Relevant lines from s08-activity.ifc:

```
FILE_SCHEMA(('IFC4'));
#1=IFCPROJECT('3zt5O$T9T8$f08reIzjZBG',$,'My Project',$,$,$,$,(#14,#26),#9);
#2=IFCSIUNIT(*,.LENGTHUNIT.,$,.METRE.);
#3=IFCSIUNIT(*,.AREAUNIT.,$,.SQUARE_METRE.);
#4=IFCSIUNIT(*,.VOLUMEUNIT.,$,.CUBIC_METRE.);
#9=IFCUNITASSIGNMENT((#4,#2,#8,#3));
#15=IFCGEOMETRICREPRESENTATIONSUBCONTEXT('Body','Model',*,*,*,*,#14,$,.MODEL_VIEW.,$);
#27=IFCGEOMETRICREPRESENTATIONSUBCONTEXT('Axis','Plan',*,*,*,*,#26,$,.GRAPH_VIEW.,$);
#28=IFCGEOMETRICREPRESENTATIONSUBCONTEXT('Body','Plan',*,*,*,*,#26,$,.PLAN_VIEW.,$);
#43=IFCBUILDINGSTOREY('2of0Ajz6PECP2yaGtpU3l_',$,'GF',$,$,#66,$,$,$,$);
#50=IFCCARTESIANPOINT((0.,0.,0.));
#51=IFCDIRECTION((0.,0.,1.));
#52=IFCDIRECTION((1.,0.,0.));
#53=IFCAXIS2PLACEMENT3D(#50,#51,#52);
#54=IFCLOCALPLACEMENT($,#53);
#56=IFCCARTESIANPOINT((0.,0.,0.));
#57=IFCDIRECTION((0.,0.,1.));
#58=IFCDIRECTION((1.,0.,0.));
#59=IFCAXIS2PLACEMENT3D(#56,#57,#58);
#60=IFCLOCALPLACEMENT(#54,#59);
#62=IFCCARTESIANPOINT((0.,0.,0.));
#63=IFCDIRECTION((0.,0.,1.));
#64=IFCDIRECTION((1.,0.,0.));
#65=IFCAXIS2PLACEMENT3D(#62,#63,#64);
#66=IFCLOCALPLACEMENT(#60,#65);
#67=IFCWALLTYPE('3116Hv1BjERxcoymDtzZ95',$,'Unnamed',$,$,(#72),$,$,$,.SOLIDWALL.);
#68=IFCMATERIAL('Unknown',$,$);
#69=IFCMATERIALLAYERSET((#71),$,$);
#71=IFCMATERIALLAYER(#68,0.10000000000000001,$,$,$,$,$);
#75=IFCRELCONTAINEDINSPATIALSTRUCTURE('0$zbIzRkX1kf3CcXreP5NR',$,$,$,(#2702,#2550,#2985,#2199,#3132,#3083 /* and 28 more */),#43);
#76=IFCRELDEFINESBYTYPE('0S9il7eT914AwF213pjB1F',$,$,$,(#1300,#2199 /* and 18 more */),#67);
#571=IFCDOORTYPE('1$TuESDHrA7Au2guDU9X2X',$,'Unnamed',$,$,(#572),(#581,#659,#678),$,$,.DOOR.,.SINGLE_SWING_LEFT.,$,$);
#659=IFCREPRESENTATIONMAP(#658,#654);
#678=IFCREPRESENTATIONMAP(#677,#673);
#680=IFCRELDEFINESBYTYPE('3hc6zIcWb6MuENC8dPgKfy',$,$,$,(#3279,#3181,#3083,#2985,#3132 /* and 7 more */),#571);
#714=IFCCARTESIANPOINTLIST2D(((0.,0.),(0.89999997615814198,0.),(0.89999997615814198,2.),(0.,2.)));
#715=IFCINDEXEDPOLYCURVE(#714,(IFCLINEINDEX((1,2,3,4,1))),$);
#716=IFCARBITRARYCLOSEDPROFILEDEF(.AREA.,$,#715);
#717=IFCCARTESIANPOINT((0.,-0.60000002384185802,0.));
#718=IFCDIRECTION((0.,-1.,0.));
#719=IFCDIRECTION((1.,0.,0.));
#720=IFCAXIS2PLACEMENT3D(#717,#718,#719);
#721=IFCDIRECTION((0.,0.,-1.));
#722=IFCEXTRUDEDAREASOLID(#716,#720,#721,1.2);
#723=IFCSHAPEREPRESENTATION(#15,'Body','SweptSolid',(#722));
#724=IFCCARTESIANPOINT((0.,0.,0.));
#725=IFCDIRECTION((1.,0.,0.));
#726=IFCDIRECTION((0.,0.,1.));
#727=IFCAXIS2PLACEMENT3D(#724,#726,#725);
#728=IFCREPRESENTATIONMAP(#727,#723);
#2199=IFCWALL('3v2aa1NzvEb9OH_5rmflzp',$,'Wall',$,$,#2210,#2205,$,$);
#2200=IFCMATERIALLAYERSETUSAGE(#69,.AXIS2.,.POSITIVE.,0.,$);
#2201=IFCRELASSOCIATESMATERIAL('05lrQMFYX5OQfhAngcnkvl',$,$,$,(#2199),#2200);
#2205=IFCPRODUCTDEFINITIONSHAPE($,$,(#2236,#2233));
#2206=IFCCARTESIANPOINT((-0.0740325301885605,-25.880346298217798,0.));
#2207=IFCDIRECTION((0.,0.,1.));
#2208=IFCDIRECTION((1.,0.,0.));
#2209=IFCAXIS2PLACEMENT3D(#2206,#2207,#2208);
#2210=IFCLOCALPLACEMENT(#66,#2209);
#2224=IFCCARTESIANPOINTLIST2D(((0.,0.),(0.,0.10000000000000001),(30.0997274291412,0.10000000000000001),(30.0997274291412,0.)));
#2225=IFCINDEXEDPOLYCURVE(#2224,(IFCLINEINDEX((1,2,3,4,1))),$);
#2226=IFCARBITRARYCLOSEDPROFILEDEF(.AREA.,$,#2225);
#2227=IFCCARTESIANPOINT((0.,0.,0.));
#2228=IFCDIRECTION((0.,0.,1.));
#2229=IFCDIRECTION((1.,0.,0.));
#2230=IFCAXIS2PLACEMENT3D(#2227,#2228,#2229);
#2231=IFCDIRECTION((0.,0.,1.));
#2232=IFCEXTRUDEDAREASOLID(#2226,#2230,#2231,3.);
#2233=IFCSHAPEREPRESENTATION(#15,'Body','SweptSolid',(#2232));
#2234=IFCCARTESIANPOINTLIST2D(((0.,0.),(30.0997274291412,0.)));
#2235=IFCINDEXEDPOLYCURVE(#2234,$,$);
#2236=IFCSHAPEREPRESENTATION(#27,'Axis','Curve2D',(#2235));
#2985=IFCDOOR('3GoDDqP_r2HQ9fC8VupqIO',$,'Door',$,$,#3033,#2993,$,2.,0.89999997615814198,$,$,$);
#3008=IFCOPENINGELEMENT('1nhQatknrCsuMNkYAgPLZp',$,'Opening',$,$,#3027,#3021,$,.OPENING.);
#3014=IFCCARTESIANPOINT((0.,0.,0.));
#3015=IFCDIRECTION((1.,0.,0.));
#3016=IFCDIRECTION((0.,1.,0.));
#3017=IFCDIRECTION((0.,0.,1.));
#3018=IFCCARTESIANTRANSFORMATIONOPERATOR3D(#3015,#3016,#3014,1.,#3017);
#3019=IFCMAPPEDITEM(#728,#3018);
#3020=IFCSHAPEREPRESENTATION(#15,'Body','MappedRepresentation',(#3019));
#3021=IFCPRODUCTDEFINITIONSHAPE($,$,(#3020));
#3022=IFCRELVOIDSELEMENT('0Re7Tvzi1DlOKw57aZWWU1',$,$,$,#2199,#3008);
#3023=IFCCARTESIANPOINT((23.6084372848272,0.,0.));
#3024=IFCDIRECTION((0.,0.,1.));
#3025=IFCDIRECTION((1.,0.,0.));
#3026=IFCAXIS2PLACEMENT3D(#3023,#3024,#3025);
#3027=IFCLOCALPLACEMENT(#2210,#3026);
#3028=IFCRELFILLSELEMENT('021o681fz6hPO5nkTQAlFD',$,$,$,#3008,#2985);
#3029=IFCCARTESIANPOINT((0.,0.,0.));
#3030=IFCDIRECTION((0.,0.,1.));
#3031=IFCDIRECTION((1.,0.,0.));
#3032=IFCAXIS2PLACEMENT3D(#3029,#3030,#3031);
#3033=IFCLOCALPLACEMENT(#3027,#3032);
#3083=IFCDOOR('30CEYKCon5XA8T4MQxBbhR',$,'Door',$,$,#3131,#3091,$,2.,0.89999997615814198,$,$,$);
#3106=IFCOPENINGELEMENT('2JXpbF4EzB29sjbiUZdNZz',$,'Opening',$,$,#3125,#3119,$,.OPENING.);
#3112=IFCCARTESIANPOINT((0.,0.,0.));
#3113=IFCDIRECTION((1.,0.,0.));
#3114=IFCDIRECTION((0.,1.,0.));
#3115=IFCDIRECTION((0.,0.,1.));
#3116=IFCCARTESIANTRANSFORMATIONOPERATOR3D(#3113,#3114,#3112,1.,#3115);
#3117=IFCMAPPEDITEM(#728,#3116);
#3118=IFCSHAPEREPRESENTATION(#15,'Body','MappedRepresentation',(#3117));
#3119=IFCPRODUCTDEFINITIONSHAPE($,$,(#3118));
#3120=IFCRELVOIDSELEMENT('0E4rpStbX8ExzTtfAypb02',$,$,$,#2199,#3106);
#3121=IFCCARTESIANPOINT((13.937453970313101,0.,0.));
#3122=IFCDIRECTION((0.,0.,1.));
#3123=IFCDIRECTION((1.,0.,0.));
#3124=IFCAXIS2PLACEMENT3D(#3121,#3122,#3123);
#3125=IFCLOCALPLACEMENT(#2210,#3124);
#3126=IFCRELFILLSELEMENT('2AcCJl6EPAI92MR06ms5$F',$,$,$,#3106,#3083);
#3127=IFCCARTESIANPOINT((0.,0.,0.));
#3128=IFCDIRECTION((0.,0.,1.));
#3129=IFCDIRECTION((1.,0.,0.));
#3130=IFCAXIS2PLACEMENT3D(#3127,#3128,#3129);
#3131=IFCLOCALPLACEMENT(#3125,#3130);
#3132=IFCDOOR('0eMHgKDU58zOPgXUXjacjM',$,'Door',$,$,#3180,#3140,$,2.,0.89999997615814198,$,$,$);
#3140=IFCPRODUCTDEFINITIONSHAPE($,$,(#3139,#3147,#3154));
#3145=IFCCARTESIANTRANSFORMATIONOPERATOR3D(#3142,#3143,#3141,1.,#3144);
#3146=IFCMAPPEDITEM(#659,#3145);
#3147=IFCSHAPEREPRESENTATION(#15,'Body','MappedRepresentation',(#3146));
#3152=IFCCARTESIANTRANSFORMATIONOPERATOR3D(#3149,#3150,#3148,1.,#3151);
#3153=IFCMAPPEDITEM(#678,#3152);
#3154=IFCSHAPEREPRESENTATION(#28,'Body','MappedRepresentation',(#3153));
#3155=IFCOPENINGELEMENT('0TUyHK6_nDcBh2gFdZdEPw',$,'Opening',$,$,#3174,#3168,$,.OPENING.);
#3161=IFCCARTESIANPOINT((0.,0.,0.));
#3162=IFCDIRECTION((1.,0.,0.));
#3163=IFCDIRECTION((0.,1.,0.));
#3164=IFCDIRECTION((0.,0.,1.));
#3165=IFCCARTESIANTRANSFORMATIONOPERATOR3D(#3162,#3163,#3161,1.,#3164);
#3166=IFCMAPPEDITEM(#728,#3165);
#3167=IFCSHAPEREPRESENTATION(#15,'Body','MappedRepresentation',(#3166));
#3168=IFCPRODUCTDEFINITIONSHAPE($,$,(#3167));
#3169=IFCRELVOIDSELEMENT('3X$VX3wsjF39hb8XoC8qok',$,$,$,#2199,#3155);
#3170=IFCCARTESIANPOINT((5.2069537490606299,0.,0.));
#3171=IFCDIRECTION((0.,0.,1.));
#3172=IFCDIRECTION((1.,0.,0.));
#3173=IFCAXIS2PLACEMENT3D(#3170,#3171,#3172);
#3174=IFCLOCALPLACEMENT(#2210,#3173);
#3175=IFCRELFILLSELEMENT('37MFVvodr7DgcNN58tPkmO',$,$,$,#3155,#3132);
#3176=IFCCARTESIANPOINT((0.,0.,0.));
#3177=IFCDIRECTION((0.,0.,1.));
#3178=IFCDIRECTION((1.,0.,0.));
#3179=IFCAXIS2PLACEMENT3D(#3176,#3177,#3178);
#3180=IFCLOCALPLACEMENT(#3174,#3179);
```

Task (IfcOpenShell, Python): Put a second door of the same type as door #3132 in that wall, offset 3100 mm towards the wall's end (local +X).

```python
import ifcopenshell
import ifcopenshell.api.feature
import ifcopenshell.api.geometry
import ifcopenshell.api.root
import ifcopenshell.geom
import ifcopenshell.util.element
import ifcopenshell.util.placement
import ifcopenshell.util.shape
import ifcopenshell.util.unit

model = ifcopenshell.open("s08-activity.ifc")
unit_scale = ifcopenshell.util.unit.calculate_unit_scale(model)
settings = ifcopenshell.geom.settings()


def volume(element):
    """Net volume in cubic metres, openings subtracted."""
    shape = ifcopenshell.geom.create_shape(settings, element)
    return ifcopenshell.util.shape.get_volume(shape.geometry)


door = model.by_guid("0eMHgKDU58zOPgXUXjacjM")
opening = door.FillsVoids[0].RelatingOpeningElement
wall = opening.VoidsElements[0].RelatingBuildingElement
before = volume(wall)
shift = ifcopenshell.util.placement.get_local_placement(wall.ObjectPlacement)[:3, 0] * 3.1 / unit_scale

# copy_class copies the void relationship, type, container and properties, but no geometry.
new_opening = ifcopenshell.api.root.copy_class(model, product=opening)
new_opening.Representation = ifcopenshell.util.element.copy_deep(
    model, opening.Representation, exclude=["IfcGeometricRepresentationContext", "IfcRepresentationMap"]
)
new_door = ifcopenshell.api.root.copy_class(model, product=door)
new_door.Representation = ifcopenshell.util.element.copy_deep(
    model, door.Representation, exclude=["IfcGeometricRepresentationContext", "IfcRepresentationMap"]
)
ifcopenshell.api.feature.add_filling(model, opening=new_opening, element=new_door)

for old, new in ((opening, new_opening), (door, new_door)):
    matrix = ifcopenshell.util.placement.get_local_placement(old.ObjectPlacement)
    matrix[:3, 3] += shift
    ifcopenshell.api.geometry.edit_object_placement(model, product=new, matrix=matrix, is_si=False)

after = volume(wall)

print(f"wall volume {before:.3f} -> {after:.3f} m3")

model.write("s08-activity_edited.ifc")
```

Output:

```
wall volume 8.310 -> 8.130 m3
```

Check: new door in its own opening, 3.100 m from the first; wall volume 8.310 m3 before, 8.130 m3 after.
